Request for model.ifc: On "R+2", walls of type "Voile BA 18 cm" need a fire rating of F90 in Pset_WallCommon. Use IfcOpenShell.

First a look at what the model holds.

```python
import ifcopenshell
import ifcopenshell.util.element

model = ifcopenshell.open("model.ifc")
print(model.schema)
storey = next(s for s in model.by_type("IfcBuildingStorey") if s.Name == "R+2")
walls = [e for e in ifcopenshell.util.element.get_decomposition(storey) if e.is_a("IfcWall")]
seen = {}
for e in walls:
    element_type = ifcopenshell.util.element.get_type(e)
    key = (element_type.Name if element_type != e and element_type else None, ifcopenshell.util.element.get_pset(e, "Pset_WallCommon", "FireRating"))
    seen[key] = seen.get(key, 0) + 1
for (name, value), count in sorted(seen.items(), key=str):
    print(count, "x", name, "|", value)
```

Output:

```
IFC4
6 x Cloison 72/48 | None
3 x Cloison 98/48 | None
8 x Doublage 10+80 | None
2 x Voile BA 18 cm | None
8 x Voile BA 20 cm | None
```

```python
import ifcopenshell
import ifcopenshell.api.pset
import ifcopenshell.util.element

model = ifcopenshell.open("model.ifc")

storey = next(s for s in model.by_type("IfcBuildingStorey") if s.Name == "R+2")
walls = [e for e in ifcopenshell.util.element.get_decomposition(storey) if e.is_a("IfcWall")]

count = 0
for e in walls:
    element_type = ifcopenshell.util.element.get_type(e)
    if element_type in (None, e) or element_type.Name != "Voile BA 18 cm":
        continue
    # add_pset returns the element's existing set when there is one.
    pset = ifcopenshell.api.pset.add_pset(model, product=e, name="Pset_WallCommon")
    ifcopenshell.api.pset.edit_pset(model, pset=pset, properties={"FireRating": "F90"})
    count += 1

print(count, "walls updated")

model.write("model_v2.ifc")
```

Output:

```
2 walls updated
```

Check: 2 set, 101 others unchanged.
